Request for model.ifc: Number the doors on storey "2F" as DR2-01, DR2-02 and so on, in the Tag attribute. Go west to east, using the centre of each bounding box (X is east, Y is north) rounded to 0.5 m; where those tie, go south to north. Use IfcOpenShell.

First a look at what the model holds.

```python
import ifcopenshell
import ifcopenshell.util.element
import ifcopenshell.util.placement

model = ifcopenshell.open("model.ifc")
print(model.schema)
storey = next(s for s in model.by_type("IfcBuildingStorey") if s.Name == "2F")
doors = [e for e in ifcopenshell.util.element.get_decomposition(storey) if e.is_a("IfcDoor")]
for e in sorted(doors, key=lambda e: e.id()):
    origin = ifcopenshell.util.placement.get_local_placement(e.ObjectPlacement)[:3, 3]
    print(e.id(), e.Tag, e.Name, origin.round(2) + 0.0, sep=" | ")
```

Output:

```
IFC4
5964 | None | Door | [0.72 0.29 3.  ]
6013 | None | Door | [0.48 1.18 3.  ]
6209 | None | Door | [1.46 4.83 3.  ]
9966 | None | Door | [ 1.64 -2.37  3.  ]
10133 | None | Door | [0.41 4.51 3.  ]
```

```python
import ifcopenshell
import ifcopenshell.geom
import ifcopenshell.util.element
import ifcopenshell.util.shape

model = ifcopenshell.open("model.ifc")
settings = ifcopenshell.geom.settings()
settings.set("use-world-coords", True)


def centre(element):
    shape = ifcopenshell.geom.create_shape(settings, element)
    return ifcopenshell.util.shape.get_bbox_centroid(shape.geometry)


storey = next(s for s in model.by_type("IfcBuildingStorey") if s.Name == "2F")
doors = [e for e in ifcopenshell.util.element.get_decomposition(storey) if e.is_a("IfcDoor")]

# Insertion points can sit at a corner or the storey origin, so sort by the geometry (in metres).
centres = {e: centre(e) for e in doors}
doors.sort(key=lambda e: (round(centres[e][0] / 0.5), centres[e][1]))

for i, e in enumerate(doors, start=1):
    number = f"DR2-{i:02d}"
    e.Tag = number
    print(e.id(), number)

model.write("model_v2.ifc")
```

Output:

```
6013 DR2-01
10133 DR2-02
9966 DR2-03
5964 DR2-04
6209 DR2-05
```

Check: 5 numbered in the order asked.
